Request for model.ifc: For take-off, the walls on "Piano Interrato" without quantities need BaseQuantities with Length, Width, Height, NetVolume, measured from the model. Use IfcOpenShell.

First a look at what the model holds.

```python
import ifcopenshell
import ifcopenshell.util.element
import ifcopenshell.util.unit

model = ifcopenshell.open("model.ifc")
print(model.schema)
for unit_type in ("LENGTHUNIT", "AREAUNIT", "VOLUMEUNIT"):
    print(unit_type, ifcopenshell.util.unit.calculate_unit_scale(model, unit_type))
storey = next(s for s in model.by_type("IfcBuildingStorey") if s.Name == "Piano Interrato")
walls = [e for e in ifcopenshell.util.element.get_decomposition(storey) if e.is_a("IfcWall")]
for e in sorted(walls, key=lambda e: e.id()):
    print(e.id(), e.is_a(), e.Name, list(ifcopenshell.util.element.get_psets(e, qtos_only=True)), sep=" | ")
```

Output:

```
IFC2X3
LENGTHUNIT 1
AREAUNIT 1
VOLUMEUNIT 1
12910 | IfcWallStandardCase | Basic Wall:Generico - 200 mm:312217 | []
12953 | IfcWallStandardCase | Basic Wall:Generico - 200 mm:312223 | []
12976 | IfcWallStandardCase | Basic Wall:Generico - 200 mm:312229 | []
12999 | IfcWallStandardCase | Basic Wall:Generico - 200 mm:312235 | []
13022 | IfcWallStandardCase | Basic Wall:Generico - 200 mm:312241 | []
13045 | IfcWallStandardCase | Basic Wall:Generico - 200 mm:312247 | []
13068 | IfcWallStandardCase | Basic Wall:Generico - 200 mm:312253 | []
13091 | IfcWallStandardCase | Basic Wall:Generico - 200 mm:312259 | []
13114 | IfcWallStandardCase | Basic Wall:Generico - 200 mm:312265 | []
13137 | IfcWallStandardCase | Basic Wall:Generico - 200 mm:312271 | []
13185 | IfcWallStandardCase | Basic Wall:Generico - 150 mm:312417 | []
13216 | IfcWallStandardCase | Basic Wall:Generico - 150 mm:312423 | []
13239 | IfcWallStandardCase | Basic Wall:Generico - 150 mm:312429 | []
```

```python
import ifcopenshell
import ifcopenshell.api.pset
import ifcopenshell.geom
import ifcopenshell.util.element
import ifcopenshell.util.shape
import ifcopenshell.util.unit

model = ifcopenshell.open("model.ifc")
unit_scale = ifcopenshell.util.unit.calculate_unit_scale(model)
volume_scale = ifcopenshell.util.unit.calculate_unit_scale(model, "VOLUMEUNIT")
settings = ifcopenshell.geom.settings()

storey = next(s for s in model.by_type("IfcBuildingStorey") if s.Name == "Piano Interrato")
walls = [e for e in ifcopenshell.util.element.get_decomposition(storey) if e.is_a("IfcWall")]

for e in sorted(walls, key=lambda e: e.id()):
    if ifcopenshell.util.element.get_psets(e, qtos_only=True, should_inherit=False):
        continue
    # Geometry comes back in metres, in the element's own axes.
    shape = ifcopenshell.geom.create_shape(settings, e)
    values = {
        "Length": ifcopenshell.util.shape.get_x(shape.geometry) / unit_scale,
        "Width": ifcopenshell.util.shape.get_y(shape.geometry) / unit_scale,
        "Height": ifcopenshell.util.shape.get_z(shape.geometry) / unit_scale,
        "NetVolume": ifcopenshell.util.shape.get_volume(shape.geometry) / volume_scale,
    }
    qto = ifcopenshell.api.pset.add_qto(model, product=e, name="BaseQuantities")
    ifcopenshell.api.pset.edit_qto(model, qto=qto, properties=values)
    print(e.id(), {k: round(v, 3) for k, v in values.items()})

model.write("model-out.ifc")
```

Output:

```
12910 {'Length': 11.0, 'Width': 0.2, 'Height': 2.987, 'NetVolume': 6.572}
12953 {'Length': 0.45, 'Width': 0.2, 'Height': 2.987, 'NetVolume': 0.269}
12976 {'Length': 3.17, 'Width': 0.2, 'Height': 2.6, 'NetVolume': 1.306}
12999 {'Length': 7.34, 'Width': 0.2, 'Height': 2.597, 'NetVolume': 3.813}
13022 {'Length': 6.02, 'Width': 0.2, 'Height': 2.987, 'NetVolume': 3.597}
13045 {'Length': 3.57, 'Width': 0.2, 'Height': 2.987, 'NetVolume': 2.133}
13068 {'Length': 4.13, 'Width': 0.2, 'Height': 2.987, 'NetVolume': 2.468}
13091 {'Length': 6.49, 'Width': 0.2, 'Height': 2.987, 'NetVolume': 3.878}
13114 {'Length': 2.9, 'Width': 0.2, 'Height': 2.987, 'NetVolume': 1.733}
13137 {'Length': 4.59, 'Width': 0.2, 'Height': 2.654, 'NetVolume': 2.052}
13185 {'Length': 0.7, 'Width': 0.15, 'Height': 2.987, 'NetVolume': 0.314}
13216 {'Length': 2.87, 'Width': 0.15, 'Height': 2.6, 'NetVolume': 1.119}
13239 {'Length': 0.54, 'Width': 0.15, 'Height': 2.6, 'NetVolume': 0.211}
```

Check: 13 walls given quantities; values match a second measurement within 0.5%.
